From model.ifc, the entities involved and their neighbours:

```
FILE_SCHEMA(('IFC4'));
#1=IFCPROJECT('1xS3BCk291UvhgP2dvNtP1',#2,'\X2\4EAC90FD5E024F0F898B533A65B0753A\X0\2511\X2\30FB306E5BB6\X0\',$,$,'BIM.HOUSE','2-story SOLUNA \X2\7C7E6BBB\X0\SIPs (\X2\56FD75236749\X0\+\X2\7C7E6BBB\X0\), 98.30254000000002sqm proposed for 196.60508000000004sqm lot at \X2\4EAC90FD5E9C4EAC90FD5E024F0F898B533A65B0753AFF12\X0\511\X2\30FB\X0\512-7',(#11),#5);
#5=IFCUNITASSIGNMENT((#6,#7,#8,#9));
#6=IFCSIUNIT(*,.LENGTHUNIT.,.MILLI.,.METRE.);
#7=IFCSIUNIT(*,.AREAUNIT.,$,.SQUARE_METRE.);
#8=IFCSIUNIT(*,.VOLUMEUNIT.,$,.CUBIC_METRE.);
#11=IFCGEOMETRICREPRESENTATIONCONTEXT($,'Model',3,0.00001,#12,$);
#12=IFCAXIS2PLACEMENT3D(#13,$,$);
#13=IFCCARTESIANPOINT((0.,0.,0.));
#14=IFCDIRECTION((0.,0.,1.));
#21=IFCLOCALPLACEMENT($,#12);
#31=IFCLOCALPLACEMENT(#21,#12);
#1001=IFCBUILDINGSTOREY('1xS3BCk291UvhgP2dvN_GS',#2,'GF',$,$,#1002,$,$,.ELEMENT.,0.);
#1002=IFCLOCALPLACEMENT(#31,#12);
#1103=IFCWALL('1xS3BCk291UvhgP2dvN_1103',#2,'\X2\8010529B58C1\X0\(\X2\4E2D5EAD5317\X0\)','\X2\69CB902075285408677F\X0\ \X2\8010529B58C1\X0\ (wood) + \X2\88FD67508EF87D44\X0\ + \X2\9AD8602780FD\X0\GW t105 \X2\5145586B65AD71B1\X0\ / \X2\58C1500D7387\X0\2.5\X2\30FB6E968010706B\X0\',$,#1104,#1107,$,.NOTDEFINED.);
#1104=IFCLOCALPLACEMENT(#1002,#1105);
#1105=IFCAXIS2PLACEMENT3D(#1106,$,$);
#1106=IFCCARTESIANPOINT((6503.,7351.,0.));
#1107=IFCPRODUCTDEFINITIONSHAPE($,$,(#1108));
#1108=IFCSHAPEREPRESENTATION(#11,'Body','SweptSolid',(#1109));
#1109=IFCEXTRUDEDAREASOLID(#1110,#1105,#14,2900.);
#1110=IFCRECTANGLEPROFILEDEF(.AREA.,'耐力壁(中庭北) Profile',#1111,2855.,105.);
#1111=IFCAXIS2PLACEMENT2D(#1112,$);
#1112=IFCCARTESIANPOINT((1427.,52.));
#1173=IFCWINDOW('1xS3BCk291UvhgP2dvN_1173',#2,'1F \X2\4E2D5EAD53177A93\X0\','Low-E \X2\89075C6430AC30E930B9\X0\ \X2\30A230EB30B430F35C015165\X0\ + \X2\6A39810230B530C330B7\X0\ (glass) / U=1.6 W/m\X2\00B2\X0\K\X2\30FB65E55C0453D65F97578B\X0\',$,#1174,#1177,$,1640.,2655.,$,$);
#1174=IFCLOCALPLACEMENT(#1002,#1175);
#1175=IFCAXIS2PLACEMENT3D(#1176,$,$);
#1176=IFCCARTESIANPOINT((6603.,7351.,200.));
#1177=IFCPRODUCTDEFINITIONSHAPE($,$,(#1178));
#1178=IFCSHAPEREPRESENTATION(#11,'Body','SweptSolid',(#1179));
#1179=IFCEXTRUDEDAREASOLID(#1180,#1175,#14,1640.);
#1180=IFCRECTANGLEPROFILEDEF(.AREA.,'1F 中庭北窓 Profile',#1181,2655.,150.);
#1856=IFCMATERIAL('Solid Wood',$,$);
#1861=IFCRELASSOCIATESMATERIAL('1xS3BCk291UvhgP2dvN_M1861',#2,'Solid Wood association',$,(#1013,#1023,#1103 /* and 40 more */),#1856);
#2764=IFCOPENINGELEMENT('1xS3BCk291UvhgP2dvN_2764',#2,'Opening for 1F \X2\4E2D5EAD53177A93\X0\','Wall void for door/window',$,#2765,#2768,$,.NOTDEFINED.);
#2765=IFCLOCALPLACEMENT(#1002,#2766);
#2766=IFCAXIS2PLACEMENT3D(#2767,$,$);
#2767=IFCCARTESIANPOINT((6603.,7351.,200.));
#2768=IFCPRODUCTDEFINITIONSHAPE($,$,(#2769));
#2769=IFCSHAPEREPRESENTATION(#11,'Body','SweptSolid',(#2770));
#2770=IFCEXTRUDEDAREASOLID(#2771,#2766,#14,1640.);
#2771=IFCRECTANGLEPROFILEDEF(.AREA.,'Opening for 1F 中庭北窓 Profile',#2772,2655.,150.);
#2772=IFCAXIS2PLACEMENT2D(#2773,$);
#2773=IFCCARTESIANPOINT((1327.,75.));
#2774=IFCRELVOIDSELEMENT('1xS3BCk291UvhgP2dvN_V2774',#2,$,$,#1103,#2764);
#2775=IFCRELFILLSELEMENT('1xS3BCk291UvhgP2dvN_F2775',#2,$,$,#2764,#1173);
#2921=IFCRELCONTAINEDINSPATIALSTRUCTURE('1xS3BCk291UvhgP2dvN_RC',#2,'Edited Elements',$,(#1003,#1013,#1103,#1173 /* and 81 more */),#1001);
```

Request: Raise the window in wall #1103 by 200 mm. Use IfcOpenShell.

```python
import numpy as np
import ifcopenshell
import ifcopenshell.api.geometry
import ifcopenshell.util.placement
import ifcopenshell.util.unit

model = ifcopenshell.open("model.ifc")
unit_scale = ifcopenshell.util.unit.calculate_unit_scale(model)

window = model.by_guid("1xS3BCk291UvhgP2dvN_1173")
opening = window.FillsVoids[0].RelatingOpeningElement
dz = 0.2 / unit_scale

shift = np.array([0.0, 0.0, dz])
# The window is not placed relative to its opening, so move both.
for product in (opening, window):
    matrix = ifcopenshell.util.placement.get_local_placement(product.ObjectPlacement)
    matrix[:3, 3] += shift
    ifcopenshell.api.geometry.edit_object_placement(model, product=product, matrix=matrix, is_si=False)

print(f"moved by {dz * unit_scale:+.3f} m")

model.write("model_updated.ifc")
```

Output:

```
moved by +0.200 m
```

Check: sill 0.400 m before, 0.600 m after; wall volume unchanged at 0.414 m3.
